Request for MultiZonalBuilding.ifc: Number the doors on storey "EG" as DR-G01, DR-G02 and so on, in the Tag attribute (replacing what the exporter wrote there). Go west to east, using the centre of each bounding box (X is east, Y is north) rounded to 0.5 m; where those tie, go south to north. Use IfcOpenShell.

First a look at what the model holds.

```python
import ifcopenshell
import ifcopenshell.util.element
import ifcopenshell.util.placement

model = ifcopenshell.open("MultiZonalBuilding.ifc")
print(model.schema)
storey = next(s for s in model.by_type("IfcBuildingStorey") if s.Name == "EG")
doors = [e for e in ifcopenshell.util.element.get_decomposition(storey) if e.is_a("IfcDoor")]
for e in sorted(doors, key=lambda e: e.id()):
    origin = ifcopenshell.util.placement.get_local_placement(e.ObjectPlacement)[:3, 3]
    print(e.id(), e.Tag, e.Name, origin.round(2) + 0.0, sep=" | ")
```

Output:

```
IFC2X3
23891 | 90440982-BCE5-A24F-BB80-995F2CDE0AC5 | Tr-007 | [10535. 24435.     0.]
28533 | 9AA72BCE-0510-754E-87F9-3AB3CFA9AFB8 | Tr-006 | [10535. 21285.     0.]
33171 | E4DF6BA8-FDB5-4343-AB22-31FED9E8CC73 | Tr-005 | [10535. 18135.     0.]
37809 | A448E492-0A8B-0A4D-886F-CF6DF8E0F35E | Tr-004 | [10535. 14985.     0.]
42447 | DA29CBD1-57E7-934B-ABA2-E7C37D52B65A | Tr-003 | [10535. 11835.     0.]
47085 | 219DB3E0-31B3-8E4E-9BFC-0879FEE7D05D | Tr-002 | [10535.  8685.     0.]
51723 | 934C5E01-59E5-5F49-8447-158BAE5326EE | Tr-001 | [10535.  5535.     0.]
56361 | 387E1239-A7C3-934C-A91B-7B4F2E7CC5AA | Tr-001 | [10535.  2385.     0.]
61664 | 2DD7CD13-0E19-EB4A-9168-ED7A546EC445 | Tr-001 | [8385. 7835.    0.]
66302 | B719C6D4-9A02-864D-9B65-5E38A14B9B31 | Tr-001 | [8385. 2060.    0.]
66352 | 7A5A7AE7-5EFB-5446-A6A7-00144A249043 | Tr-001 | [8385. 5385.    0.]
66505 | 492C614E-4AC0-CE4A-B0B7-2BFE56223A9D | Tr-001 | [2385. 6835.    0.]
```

```python
import ifcopenshell
import ifcopenshell.geom
import ifcopenshell.util.element
import ifcopenshell.util.shape

model = ifcopenshell.open("MultiZonalBuilding.ifc")
settings = ifcopenshell.geom.settings()
settings.set("use-world-coords", True)


def centre(element):
    shape = ifcopenshell.geom.create_shape(settings, element)
    return ifcopenshell.util.shape.get_bbox_centroid(shape.geometry)


storey = next(s for s in model.by_type("IfcBuildingStorey") if s.Name == "EG")
doors = [e for e in ifcopenshell.util.element.get_decomposition(storey) if e.is_a("IfcDoor")]

# Insertion points can sit at a corner or the storey origin, so sort by the geometry (in metres).
centres = {e: centre(e) for e in doors}
doors.sort(key=lambda e: (round(centres[e][0] / 0.5), centres[e][1]))

for i, e in enumerate(doors, start=1):
    number = f"DR-G{i:02d}"
    e.Tag = number
    print(e.id(), number)

model.write("MultiZonalBuilding_v2.ifc")
```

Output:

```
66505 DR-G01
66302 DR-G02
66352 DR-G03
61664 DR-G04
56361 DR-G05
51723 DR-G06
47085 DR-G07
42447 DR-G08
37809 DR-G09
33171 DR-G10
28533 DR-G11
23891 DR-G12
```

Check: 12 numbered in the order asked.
